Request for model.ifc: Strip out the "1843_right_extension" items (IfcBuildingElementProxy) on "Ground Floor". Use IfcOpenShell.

First a look at what the model holds.

```python
import ifcopenshell
import ifcopenshell.util.element

model = ifcopenshell.open("model.ifc")
print(model.schema)
storey = next(s for s in model.by_type("IfcBuildingStorey") if s.Name == "Ground Floor")
proxies = [e for e in ifcopenshell.util.element.get_decomposition(storey) if e.is_a("IfcBuildingElementProxy")]
seen = {}
for e in proxies:
    element_type = ifcopenshell.util.element.get_type(e)
    name = element_type.Name if element_type not in (None, e) else None
    seen[name] = seen.get(name, 0) + 1
for name, count in sorted(seen.items(), key=str):
    print(count, "x", name)
```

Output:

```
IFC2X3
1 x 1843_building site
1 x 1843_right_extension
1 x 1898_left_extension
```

```python
import ifcopenshell
import ifcopenshell.api.root
import ifcopenshell.util.element

model = ifcopenshell.open("model.ifc")

storey = next(s for s in model.by_type("IfcBuildingStorey") if s.Name == "Ground Floor")
proxies = [e for e in ifcopenshell.util.element.get_decomposition(storey) if e.is_a("IfcBuildingElementProxy")]
targets = [e for e in proxies if (t := ifcopenshell.util.element.get_type(e)) not in (None, e) and t.Name == "1843_right_extension"]

for e in targets:
    ifcopenshell.api.root.remove_product(model, product=e)
print(len(targets), "removed")

model.write("model_updated.ifc")
```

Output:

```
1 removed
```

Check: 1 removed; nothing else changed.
